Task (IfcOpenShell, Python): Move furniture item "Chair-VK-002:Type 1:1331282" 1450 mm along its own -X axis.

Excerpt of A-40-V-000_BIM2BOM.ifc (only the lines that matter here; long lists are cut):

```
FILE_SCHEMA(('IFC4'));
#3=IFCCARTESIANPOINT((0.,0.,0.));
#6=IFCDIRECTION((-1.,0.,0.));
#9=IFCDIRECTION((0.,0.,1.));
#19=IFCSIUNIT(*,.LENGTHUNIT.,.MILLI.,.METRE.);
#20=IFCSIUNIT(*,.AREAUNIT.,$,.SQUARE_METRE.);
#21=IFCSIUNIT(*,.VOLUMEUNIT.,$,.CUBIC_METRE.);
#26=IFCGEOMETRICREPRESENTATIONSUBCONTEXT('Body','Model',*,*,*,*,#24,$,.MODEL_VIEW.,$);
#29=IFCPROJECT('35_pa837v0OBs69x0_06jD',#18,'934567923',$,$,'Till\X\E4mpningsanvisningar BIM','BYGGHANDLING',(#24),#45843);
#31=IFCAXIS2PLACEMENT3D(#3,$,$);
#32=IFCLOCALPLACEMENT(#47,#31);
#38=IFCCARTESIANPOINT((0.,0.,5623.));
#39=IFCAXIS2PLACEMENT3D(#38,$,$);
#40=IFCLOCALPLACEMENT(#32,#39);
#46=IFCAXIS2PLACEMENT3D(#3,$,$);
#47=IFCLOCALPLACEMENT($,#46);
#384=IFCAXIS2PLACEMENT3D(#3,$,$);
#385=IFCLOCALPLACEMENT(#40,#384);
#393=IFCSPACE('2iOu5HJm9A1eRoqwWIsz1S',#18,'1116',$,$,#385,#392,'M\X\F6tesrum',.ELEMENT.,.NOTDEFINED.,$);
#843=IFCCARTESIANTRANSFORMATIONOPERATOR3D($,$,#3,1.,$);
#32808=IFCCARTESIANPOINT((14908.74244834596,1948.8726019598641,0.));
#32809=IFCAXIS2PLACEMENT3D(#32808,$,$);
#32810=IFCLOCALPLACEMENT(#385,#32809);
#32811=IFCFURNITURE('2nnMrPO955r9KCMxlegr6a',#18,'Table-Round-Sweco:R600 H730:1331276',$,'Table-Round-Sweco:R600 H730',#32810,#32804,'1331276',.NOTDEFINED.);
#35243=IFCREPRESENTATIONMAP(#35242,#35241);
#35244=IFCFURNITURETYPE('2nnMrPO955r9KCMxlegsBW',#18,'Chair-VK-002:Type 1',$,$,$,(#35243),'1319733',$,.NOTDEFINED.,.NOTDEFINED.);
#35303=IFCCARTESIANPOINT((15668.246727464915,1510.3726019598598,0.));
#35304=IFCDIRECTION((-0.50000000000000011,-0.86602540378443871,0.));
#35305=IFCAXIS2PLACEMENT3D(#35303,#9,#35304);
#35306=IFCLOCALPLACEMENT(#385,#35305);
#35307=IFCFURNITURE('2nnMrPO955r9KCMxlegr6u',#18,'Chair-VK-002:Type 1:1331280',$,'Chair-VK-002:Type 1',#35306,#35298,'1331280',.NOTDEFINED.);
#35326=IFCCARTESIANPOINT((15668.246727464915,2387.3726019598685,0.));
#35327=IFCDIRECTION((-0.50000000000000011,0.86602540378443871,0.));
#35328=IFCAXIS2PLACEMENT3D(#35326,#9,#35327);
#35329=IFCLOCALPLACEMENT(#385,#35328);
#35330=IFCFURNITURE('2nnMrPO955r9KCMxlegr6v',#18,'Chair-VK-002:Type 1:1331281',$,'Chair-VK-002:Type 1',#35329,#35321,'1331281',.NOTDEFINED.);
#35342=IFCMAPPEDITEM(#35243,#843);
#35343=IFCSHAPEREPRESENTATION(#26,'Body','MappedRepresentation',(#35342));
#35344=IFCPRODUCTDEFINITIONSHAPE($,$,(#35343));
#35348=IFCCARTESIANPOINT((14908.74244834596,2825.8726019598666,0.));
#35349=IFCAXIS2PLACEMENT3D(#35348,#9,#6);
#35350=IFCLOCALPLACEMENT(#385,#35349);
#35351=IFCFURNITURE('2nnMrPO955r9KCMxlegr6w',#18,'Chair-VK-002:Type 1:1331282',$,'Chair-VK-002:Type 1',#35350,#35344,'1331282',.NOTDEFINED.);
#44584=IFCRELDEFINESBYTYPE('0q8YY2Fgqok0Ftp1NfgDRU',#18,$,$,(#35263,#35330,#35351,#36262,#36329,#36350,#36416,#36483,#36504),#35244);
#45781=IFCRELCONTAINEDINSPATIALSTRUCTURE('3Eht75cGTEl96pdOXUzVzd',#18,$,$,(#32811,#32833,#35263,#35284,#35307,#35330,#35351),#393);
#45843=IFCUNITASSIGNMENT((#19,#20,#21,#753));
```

```python
import ifcopenshell
import ifcopenshell.api.geometry
import ifcopenshell.util.placement

model = ifcopenshell.open("A-40-V-000_BIM2BOM.ifc")

item = model.by_id(35351)
matrix = ifcopenshell.util.placement.get_local_placement(item.ObjectPlacement)
matrix[:3, 3] -= matrix[:3, 0] * 1450.0
ifcopenshell.api.geometry.edit_object_placement(model, product=item, matrix=matrix, is_si=False)

print(ifcopenshell.util.placement.get_local_placement(item.ObjectPlacement).round(3) + 0.0)

model.write("A-40-V-000_BIM2BOM_updated.ifc")
```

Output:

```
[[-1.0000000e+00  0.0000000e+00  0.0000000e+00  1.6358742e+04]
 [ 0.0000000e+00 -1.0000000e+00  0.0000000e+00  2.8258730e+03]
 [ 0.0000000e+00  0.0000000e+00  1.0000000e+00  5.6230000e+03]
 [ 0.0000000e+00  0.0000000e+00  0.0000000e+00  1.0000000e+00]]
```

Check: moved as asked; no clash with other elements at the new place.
